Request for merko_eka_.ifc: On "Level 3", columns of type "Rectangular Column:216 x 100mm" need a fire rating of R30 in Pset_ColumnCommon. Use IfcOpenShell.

First a look at what the model holds.

```python
import ifcopenshell
import ifcopenshell.util.element

model = ifcopenshell.open("merko_eka_.ifc")
print(model.schema)
storey = next(s for s in model.by_type("IfcBuildingStorey") if s.Name == "Level 3")
columns = [e for e in ifcopenshell.util.element.get_decomposition(storey) if e.is_a("IfcColumn")]
seen = {}
for e in columns:
    element_type = ifcopenshell.util.element.get_type(e)
    key = (element_type.Name if element_type != e and element_type else None, ifcopenshell.util.element.get_pset(e, "Pset_ColumnCommon", "FireRating"))
    seen[key] = seen.get(key, 0) + 1
for (name, value), count in sorted(seen.items(), key=str):
    print(count, "x", name, "|", value)
```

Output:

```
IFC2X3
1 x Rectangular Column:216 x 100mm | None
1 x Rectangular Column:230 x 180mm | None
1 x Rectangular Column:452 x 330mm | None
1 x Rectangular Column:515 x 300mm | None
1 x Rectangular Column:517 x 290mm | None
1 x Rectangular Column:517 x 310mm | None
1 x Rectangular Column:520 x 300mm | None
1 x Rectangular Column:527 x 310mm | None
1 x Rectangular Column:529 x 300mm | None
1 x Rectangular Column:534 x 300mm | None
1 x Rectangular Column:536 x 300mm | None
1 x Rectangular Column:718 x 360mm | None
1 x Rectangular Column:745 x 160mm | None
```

```python
import ifcopenshell
import ifcopenshell.api.pset
import ifcopenshell.util.element

model = ifcopenshell.open("merko_eka_.ifc")

storey = next(s for s in model.by_type("IfcBuildingStorey") if s.Name == "Level 3")
columns = [e for e in ifcopenshell.util.element.get_decomposition(storey) if e.is_a("IfcColumn")]

count = 0
for e in columns:
    element_type = ifcopenshell.util.element.get_type(e)
    if element_type in (None, e) or element_type.Name != "Rectangular Column:216 x 100mm":
        continue
    # add_pset returns the element's existing set when there is one.
    pset = ifcopenshell.api.pset.add_pset(model, product=e, name="Pset_ColumnCommon")
    ifcopenshell.api.pset.edit_pset(model, pset=pset, properties={"FireRating": "R30"})
    count += 1

print(count, "columns updated")

model.write("merko_eka__edited.ifc")
```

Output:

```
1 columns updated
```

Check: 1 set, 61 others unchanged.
